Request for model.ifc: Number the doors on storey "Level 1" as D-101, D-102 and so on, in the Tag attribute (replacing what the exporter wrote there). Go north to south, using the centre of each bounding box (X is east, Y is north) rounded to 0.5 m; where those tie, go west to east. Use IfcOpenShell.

First a look at what the model holds.

```python
import ifcopenshell
import ifcopenshell.util.element
import ifcopenshell.util.placement

model = ifcopenshell.open("model.ifc")
print(model.schema)
storey = next(s for s in model.by_type("IfcBuildingStorey") if s.Name == "Level 1")
doors = [e for e in ifcopenshell.util.element.get_decomposition(storey) if e.is_a("IfcDoor")]
for e in sorted(doors, key=lambda e: e.id()):
    origin = ifcopenshell.util.placement.get_local_placement(e.ObjectPlacement)[:3, 3]
    print(e.id(), e.Tag, e.Name, origin.round(2) + 0.0, sep=" | ")
```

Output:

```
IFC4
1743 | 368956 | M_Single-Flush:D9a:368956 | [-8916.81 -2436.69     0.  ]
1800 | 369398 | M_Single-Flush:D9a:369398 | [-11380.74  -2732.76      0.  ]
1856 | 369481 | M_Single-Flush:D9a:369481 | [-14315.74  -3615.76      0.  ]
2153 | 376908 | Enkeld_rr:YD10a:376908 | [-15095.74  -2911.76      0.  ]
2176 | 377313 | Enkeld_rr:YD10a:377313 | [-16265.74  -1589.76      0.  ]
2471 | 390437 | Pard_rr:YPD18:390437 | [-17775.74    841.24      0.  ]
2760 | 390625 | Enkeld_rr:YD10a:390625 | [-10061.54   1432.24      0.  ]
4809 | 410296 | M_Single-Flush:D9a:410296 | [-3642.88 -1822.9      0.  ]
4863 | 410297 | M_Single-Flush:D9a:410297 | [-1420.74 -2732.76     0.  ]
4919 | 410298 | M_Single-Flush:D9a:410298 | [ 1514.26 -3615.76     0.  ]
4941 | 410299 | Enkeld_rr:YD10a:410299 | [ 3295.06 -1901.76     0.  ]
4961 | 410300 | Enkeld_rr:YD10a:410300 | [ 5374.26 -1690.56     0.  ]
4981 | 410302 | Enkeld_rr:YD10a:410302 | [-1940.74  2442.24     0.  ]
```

```python
import ifcopenshell
import ifcopenshell.geom
import ifcopenshell.util.element
import ifcopenshell.util.shape

model = ifcopenshell.open("model.ifc")
settings = ifcopenshell.geom.settings()
settings.set("use-world-coords", True)


def centre(element):
    shape = ifcopenshell.geom.create_shape(settings, element)
    return ifcopenshell.util.shape.get_bbox_centroid(shape.geometry)


storey = next(s for s in model.by_type("IfcBuildingStorey") if s.Name == "Level 1")
doors = [e for e in ifcopenshell.util.element.get_decomposition(storey) if e.is_a("IfcDoor")]

# Insertion points can sit at a corner or the storey origin, so sort by the geometry (in metres).
centres = {e: centre(e) for e in doors}
doors.sort(key=lambda e: (-round(centres[e][1] / 0.5), centres[e][0]))

for i, e in enumerate(doors, start=1):
    number = f"D-1{i:02d}"
    e.Tag = number
    print(e.id(), number)

model.write("model_edited.ifc")
```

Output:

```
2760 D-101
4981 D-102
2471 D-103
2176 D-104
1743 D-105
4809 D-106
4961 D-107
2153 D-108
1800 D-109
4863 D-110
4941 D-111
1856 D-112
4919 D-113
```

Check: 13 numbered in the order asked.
